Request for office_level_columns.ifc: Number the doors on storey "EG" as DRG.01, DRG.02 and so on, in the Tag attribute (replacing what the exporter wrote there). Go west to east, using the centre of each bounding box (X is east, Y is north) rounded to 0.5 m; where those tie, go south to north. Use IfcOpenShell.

First a look at what the model holds.

```python
import ifcopenshell
import ifcopenshell.util.element
import ifcopenshell.util.placement

model = ifcopenshell.open("office_level_columns.ifc")
print(model.schema)
storey = next(s for s in model.by_type("IfcBuildingStorey") if s.Name == "EG")
doors = [e for e in ifcopenshell.util.element.get_decomposition(storey) if e.is_a("IfcDoor")]
for e in sorted(doors, key=lambda e: e.id()):
    origin = ifcopenshell.util.placement.get_local_placement(e.ObjectPlacement)[:3, 3]
    print(e.id(), e.Tag, e.Name, origin.round(2) + 0.0, sep=" | ")
```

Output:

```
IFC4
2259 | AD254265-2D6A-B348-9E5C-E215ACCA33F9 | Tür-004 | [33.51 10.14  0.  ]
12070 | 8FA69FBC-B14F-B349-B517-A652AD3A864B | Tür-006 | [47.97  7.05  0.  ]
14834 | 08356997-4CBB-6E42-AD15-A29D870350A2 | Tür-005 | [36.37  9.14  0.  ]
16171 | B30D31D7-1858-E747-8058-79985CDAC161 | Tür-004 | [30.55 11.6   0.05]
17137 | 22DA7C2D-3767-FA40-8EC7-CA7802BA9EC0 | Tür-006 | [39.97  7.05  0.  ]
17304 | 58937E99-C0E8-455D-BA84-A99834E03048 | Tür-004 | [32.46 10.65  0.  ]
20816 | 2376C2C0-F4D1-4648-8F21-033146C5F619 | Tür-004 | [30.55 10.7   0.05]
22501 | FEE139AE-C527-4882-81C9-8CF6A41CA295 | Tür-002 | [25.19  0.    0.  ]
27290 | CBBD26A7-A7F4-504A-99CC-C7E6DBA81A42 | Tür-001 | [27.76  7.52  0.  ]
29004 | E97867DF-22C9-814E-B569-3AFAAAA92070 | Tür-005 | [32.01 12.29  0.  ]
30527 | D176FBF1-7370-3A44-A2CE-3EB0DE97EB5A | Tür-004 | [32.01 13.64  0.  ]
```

```python
import ifcopenshell
import ifcopenshell.geom
import ifcopenshell.util.element
import ifcopenshell.util.shape

model = ifcopenshell.open("office_level_columns.ifc")
settings = ifcopenshell.geom.settings()
settings.set("use-world-coords", True)


def centre(element):
    shape = ifcopenshell.geom.create_shape(settings, element)
    return ifcopenshell.util.shape.get_bbox_centroid(shape.geometry)


storey = next(s for s in model.by_type("IfcBuildingStorey") if s.Name == "EG")
doors = [e for e in ifcopenshell.util.element.get_decomposition(storey) if e.is_a("IfcDoor")]

# Insertion points can sit at a corner or the storey origin, so sort by the geometry (in metres).
centres = {e: centre(e) for e in doors}
doors.sort(key=lambda e: (round(centres[e][0] / 0.5), centres[e][1]))

for i, e in enumerate(doors, start=1):
    number = f"DRG.{i:02d}"
    e.Tag = number
    print(e.id(), number)

model.write("office_level_columns-out.ifc")
```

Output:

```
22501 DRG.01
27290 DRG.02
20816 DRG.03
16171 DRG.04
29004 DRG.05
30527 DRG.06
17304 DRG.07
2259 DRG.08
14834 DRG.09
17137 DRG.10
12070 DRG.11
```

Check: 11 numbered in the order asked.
